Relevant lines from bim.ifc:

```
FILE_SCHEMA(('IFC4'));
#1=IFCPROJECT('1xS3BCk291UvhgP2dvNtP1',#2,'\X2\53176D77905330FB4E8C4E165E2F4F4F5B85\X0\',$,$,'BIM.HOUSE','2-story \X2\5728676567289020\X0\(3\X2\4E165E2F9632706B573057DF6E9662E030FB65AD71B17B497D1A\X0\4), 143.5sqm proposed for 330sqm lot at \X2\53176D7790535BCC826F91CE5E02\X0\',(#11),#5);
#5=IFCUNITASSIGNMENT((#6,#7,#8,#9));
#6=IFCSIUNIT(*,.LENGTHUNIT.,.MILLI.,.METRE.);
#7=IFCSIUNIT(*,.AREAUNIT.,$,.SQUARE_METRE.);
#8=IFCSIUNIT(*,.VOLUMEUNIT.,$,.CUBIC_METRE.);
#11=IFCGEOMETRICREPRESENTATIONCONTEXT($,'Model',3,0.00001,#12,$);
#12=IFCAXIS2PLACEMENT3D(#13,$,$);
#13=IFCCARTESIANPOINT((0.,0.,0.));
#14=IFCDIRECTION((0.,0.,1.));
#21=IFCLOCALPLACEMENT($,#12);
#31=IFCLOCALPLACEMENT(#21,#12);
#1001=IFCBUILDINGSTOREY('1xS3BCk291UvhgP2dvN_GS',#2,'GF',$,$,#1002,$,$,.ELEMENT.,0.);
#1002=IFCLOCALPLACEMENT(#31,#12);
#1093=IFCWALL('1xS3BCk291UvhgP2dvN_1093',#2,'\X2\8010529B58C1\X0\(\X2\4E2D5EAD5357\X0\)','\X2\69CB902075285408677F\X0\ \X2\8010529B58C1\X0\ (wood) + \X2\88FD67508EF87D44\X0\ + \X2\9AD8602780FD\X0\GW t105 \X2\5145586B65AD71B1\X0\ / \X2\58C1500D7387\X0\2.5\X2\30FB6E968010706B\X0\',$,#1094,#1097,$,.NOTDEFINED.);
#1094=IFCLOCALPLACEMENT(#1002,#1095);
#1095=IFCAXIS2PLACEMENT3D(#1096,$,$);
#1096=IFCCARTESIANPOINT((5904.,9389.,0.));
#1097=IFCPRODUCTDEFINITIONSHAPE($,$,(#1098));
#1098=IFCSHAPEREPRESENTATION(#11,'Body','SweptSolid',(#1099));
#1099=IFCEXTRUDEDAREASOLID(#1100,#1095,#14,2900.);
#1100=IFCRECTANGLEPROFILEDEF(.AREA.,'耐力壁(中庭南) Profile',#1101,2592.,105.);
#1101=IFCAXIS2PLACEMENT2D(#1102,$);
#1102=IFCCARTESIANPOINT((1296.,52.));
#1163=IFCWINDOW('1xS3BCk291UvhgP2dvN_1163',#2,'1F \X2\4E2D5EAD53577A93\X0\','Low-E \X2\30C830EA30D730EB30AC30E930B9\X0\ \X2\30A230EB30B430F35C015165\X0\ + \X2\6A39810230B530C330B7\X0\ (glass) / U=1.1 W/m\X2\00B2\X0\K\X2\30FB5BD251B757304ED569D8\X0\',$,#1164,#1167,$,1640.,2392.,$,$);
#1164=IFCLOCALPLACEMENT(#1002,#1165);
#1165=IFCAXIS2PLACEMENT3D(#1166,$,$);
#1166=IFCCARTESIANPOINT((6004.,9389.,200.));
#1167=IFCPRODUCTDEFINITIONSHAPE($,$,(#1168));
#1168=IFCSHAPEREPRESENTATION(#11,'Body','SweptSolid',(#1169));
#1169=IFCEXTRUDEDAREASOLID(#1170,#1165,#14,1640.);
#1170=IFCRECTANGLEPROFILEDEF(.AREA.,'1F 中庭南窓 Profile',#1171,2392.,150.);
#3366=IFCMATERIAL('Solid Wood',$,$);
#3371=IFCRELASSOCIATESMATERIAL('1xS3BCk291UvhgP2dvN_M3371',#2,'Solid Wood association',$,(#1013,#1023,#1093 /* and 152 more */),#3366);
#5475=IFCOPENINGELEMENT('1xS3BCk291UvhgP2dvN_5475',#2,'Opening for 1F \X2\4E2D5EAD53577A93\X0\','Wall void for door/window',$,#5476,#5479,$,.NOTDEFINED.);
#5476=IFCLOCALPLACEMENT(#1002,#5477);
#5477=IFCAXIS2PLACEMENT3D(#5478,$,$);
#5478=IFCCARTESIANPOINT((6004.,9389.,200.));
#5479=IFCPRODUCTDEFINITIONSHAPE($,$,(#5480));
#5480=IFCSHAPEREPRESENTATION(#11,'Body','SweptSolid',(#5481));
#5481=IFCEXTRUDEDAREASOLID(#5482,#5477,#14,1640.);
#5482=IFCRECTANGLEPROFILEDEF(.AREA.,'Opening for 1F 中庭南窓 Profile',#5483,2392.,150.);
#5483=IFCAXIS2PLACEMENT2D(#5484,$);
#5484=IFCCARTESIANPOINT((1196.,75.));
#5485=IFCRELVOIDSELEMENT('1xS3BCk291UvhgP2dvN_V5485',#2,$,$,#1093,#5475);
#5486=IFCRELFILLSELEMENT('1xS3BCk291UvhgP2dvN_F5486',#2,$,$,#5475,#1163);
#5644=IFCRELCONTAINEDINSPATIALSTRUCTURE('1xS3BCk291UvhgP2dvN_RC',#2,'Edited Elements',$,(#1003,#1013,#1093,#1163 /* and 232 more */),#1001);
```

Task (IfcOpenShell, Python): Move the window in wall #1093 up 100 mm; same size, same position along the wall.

```python
import numpy as np
import ifcopenshell
import ifcopenshell.api.geometry
import ifcopenshell.util.placement
import ifcopenshell.util.unit

model = ifcopenshell.open("bim.ifc")
unit_scale = ifcopenshell.util.unit.calculate_unit_scale(model)

window = model.by_guid("1xS3BCk291UvhgP2dvN_1163")
opening = window.FillsVoids[0].RelatingOpeningElement
dz = 0.1 / unit_scale

shift = np.array([0.0, 0.0, dz])
# The window is not placed relative to its opening, so move both.
for product in (opening, window):
    matrix = ifcopenshell.util.placement.get_local_placement(product.ObjectPlacement)
    matrix[:3, 3] += shift
    ifcopenshell.api.geometry.edit_object_placement(model, product=product, matrix=matrix, is_si=False)

print(f"moved by {dz * unit_scale:+.3f} m")

model.write("bim_updated.ifc")
```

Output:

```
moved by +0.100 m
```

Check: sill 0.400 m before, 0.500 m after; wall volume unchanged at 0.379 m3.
